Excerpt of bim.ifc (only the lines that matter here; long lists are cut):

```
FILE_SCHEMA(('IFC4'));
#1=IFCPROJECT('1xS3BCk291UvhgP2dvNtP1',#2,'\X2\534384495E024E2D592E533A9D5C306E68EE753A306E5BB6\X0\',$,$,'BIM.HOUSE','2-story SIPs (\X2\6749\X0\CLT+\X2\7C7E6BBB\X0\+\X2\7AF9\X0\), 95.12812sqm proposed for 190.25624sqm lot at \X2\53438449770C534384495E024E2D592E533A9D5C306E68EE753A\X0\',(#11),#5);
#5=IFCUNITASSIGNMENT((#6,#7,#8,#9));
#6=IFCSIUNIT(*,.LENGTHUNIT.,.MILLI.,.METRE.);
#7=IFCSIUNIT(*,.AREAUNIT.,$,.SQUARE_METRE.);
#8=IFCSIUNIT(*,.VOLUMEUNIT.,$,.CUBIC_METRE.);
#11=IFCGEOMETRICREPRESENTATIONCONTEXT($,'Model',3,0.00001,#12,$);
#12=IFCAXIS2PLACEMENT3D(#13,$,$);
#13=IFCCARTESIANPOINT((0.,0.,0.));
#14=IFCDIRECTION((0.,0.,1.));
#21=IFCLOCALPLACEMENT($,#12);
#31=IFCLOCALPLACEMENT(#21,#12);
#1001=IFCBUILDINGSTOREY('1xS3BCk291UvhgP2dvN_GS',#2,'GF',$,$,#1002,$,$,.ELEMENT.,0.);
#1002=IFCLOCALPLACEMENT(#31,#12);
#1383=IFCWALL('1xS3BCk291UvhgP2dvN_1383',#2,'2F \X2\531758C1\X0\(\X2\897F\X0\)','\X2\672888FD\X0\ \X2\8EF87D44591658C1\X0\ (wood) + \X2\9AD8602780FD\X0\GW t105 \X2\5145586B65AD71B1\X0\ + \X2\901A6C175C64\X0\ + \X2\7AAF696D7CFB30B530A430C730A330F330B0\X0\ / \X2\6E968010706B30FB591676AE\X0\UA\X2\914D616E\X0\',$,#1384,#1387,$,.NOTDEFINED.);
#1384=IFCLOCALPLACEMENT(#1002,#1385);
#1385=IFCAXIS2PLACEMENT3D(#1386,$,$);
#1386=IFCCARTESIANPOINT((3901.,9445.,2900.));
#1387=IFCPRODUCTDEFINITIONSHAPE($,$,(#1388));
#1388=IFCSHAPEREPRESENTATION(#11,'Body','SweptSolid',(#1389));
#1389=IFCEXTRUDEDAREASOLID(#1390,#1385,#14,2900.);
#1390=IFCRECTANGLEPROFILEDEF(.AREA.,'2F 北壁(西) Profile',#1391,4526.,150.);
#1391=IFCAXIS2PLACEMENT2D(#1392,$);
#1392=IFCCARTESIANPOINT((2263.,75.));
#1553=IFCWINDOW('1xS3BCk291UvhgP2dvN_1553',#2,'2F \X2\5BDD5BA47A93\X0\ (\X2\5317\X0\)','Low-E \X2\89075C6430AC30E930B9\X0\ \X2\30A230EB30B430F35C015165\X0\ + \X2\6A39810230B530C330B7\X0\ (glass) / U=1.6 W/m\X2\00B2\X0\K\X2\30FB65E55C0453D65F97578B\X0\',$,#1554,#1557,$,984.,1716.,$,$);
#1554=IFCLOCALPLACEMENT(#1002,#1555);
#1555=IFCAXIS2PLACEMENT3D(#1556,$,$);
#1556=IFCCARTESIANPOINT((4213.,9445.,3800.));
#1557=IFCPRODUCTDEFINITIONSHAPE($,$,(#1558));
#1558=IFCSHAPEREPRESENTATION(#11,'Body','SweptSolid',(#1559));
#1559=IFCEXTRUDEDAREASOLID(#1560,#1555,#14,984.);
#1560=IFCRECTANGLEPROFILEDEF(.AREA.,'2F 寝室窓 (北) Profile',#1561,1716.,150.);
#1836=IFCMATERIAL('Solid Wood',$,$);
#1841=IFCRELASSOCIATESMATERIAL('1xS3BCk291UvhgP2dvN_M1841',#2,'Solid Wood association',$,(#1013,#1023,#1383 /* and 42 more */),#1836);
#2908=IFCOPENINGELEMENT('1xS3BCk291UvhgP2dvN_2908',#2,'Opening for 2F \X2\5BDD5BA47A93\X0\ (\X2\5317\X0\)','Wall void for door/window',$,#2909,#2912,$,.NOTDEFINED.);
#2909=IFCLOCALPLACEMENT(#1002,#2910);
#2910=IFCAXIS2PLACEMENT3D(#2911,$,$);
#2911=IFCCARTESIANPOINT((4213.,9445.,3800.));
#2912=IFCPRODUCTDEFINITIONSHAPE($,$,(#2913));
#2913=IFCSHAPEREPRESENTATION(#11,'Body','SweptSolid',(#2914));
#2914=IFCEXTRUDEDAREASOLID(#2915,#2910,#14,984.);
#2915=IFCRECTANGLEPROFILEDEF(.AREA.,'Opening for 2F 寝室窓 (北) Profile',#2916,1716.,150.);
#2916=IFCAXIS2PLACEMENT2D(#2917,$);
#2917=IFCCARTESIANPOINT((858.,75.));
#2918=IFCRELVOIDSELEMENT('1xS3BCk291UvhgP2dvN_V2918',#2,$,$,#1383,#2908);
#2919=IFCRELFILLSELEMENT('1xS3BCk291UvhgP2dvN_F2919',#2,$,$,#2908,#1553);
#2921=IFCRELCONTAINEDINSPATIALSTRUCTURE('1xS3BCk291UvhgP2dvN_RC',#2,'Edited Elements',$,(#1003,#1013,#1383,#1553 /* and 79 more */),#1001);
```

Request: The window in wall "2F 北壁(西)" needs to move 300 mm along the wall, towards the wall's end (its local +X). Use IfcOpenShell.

```python
import ifcopenshell
import ifcopenshell.api.geometry
import ifcopenshell.util.placement

model = ifcopenshell.open("bim.ifc")

window = model.by_guid("1xS3BCk291UvhgP2dvN_1553")
opening = window.FillsVoids[0].RelatingOpeningElement
wall = opening.VoidsElements[0].RelatingBuildingElement

wall_matrix = ifcopenshell.util.placement.get_local_placement(wall.ObjectPlacement)
shift = wall_matrix[:3, 0] * 300.0
before = ifcopenshell.util.placement.get_local_placement(window.ObjectPlacement)[:3, 3].copy()

# The window is not placed relative to its opening, so move both.
for product in (opening, window):
    matrix = ifcopenshell.util.placement.get_local_placement(product.ObjectPlacement)
    matrix[:3, 3] += shift
    ifcopenshell.api.geometry.edit_object_placement(model, product=product, matrix=matrix, is_si=False)

after = ifcopenshell.util.placement.get_local_placement(window.ObjectPlacement)[:3, 3]
print("window moved by", (after - before).round(3) + 0.0)

model.write("bim_v2.ifc")
```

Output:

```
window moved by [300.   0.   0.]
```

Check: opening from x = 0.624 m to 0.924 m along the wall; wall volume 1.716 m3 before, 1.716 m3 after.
